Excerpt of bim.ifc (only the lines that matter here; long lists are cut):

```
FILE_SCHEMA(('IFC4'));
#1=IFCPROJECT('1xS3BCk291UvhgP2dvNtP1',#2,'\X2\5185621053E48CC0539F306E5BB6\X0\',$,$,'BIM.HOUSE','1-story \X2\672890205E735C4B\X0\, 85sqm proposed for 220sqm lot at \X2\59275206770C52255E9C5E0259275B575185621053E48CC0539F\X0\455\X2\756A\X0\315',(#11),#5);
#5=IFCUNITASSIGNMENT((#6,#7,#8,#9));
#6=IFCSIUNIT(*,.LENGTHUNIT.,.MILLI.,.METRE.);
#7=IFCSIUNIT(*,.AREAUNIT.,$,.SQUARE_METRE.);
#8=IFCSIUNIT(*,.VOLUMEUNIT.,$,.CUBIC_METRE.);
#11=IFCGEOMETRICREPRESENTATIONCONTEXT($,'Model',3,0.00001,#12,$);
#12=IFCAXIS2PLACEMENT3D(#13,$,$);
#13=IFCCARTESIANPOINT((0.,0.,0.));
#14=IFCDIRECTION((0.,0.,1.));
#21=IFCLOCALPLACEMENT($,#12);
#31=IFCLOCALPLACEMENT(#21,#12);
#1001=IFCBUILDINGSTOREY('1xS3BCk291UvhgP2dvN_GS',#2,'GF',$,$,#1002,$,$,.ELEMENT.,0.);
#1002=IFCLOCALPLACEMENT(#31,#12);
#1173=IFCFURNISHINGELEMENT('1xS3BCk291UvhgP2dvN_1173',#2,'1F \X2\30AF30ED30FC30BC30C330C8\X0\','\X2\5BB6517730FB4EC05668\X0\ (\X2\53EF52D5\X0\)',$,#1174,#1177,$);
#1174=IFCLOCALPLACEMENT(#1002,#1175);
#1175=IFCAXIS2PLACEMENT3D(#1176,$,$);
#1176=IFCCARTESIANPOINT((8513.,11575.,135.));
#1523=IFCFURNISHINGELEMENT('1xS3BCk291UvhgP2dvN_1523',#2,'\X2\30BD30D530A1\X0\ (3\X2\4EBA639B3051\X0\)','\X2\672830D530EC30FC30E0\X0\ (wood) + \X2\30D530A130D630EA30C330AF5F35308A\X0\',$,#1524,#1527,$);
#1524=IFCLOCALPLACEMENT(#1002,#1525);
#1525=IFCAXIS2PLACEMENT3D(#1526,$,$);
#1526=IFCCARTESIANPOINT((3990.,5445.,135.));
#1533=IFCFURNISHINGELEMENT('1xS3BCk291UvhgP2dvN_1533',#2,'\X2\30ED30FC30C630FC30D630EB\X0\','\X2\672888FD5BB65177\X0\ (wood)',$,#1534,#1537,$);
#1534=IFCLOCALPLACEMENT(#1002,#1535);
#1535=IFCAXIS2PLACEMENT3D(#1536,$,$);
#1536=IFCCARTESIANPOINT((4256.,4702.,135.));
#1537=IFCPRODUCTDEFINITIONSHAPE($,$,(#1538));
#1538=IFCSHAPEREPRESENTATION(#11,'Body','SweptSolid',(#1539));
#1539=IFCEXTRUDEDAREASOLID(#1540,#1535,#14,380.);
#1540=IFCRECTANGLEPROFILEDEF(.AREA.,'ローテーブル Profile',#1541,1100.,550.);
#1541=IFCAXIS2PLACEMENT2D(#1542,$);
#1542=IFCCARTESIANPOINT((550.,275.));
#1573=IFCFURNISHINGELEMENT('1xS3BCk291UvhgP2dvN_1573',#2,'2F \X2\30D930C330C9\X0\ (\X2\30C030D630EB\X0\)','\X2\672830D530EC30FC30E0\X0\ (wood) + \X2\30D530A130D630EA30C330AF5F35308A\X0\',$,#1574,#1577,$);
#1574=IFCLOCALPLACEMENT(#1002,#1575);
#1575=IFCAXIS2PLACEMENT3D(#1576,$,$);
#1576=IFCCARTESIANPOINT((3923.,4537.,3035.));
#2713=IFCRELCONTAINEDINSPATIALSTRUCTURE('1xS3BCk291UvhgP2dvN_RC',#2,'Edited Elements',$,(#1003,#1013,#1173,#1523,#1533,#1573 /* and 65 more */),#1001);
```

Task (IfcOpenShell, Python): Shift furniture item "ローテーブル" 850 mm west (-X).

```python
import ifcopenshell
import ifcopenshell.api.geometry
import ifcopenshell.util.placement

model = ifcopenshell.open("bim.ifc")

item = model.by_guid("1xS3BCk291UvhgP2dvN_1533")
matrix = ifcopenshell.util.placement.get_local_placement(item.ObjectPlacement)
matrix[0, 3] -= 850.0
ifcopenshell.api.geometry.edit_object_placement(model, product=item, matrix=matrix, is_si=False)

print(ifcopenshell.util.placement.get_local_placement(item.ObjectPlacement).round(3) + 0.0)

model.write("bim_rev.ifc")
```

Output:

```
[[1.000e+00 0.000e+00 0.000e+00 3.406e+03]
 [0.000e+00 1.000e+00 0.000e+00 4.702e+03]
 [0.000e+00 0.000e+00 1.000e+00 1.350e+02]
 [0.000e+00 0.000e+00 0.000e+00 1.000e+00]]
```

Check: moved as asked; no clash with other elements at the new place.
